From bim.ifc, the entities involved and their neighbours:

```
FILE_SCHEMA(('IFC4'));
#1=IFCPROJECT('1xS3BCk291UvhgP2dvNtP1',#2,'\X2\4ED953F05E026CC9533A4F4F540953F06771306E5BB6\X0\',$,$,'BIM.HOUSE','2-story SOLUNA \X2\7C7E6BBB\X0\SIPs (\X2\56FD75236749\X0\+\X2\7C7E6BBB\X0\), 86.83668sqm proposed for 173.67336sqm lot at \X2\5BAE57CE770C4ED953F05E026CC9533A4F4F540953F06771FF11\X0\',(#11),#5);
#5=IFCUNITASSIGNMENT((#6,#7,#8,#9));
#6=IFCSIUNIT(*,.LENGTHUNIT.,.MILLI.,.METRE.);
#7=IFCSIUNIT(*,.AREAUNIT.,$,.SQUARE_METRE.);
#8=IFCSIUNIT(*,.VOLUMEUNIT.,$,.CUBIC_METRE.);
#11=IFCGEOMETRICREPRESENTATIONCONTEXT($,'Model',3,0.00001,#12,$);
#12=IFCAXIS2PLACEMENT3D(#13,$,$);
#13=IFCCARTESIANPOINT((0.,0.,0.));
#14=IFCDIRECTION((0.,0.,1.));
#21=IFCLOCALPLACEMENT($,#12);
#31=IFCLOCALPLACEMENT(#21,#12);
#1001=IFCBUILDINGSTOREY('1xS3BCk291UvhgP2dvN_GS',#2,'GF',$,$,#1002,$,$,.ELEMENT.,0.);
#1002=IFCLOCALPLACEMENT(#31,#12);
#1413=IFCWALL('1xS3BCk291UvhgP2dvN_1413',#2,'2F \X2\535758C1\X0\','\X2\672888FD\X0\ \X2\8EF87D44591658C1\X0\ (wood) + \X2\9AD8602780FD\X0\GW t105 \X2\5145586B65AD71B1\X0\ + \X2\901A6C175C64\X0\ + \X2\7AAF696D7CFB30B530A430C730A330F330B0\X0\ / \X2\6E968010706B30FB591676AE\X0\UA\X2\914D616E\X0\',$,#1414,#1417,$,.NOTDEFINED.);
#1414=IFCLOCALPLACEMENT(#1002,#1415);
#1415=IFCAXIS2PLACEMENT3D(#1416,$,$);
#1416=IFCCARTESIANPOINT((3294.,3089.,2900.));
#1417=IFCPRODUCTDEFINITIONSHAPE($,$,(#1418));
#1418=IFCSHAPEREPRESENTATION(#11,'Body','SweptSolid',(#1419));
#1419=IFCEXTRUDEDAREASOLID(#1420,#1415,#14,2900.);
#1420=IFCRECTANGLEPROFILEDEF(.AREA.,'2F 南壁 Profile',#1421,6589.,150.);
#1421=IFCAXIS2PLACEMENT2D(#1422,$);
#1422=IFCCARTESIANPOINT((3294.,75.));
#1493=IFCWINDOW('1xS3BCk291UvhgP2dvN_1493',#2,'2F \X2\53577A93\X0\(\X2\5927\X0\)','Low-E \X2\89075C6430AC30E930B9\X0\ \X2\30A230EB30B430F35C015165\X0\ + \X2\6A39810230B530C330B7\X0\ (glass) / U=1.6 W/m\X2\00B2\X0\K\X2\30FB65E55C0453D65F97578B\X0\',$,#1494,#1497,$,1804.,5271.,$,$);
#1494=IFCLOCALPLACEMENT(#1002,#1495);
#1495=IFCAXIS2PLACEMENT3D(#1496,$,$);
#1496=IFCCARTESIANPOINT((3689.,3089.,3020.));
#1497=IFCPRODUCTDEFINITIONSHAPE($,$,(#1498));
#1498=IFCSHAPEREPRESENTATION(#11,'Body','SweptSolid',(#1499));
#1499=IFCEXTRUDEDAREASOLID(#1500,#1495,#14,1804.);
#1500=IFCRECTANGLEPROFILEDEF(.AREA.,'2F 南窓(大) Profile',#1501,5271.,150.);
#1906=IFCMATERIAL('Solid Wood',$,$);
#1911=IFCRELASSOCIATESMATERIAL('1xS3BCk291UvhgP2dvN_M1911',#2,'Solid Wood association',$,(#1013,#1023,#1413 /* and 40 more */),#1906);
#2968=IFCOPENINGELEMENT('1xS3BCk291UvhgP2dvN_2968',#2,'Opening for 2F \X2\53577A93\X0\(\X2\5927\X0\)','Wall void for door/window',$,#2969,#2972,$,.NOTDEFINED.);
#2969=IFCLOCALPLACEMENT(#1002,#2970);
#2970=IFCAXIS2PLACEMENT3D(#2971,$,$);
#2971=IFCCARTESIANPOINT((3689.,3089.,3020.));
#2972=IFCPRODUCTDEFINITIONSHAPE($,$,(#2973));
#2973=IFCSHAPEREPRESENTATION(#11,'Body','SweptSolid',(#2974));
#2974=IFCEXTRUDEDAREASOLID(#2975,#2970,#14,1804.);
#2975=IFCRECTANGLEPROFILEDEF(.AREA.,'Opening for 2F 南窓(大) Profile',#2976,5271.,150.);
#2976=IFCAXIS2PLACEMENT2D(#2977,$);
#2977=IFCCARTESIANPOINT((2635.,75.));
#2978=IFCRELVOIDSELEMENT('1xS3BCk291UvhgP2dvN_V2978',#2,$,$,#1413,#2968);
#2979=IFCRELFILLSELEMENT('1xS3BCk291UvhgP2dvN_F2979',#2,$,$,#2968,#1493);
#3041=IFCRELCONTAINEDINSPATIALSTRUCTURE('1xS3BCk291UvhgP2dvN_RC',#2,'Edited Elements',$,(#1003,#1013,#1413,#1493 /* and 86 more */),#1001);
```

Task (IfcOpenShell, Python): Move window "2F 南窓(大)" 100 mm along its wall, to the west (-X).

```python
import ifcopenshell
import ifcopenshell.api.geometry
import ifcopenshell.util.placement
import ifcopenshell.util.unit

model = ifcopenshell.open("bim.ifc")
unit_scale = ifcopenshell.util.unit.calculate_unit_scale(model)

window = model.by_guid("1xS3BCk291UvhgP2dvN_1493")
opening = window.FillsVoids[0].RelatingOpeningElement
wall = opening.VoidsElements[0].RelatingBuildingElement

wall_matrix = ifcopenshell.util.placement.get_local_placement(wall.ObjectPlacement)
shift = wall_matrix[:3, 0] * -0.1 / unit_scale
before = ifcopenshell.util.placement.get_local_placement(window.ObjectPlacement)[:3, 3].copy()

# The window is not placed relative to its opening, so move both.
for product in (opening, window):
    matrix = ifcopenshell.util.placement.get_local_placement(product.ObjectPlacement)
    matrix[:3, 3] += shift
    ifcopenshell.api.geometry.edit_object_placement(model, product=product, matrix=matrix, is_si=False)

after = ifcopenshell.util.placement.get_local_placement(window.ObjectPlacement)[:3, 3]
print("window moved by", (after - before).round(3) + 0.0)

model.write("bim-out.ifc")
```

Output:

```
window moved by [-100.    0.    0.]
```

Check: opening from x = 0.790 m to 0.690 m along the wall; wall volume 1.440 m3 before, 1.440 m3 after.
